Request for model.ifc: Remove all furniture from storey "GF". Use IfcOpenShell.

First a look at what the model holds.

```python
import ifcopenshell
import ifcopenshell.util.element

model = ifcopenshell.open("model.ifc")
print(model.schema)
storey = next(s for s in model.by_type("IfcBuildingStorey") if s.Name == "GF")
furniture = [e for e in ifcopenshell.util.element.get_decomposition(storey) if e.is_a("IfcFurnishingElement")]
seen = {}
for e in furniture:
    element_type = ifcopenshell.util.element.get_type(e)
    name = element_type.Name if element_type not in (None, e) else None
    seen[name] = seen.get(name, 0) + 1
for name, count in sorted(seen.items(), key=str):
    print(count, "x", name)
```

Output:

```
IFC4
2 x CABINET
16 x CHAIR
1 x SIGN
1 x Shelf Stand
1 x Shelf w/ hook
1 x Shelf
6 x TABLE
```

```python
import ifcopenshell
import ifcopenshell.api.root
import ifcopenshell.util.element

model = ifcopenshell.open("model.ifc")

storey = next(s for s in model.by_type("IfcBuildingStorey") if s.Name == "GF")
furniture = [e for e in ifcopenshell.util.element.get_decomposition(storey) if e.is_a("IfcFurnishingElement")]

for e in furniture:
    ifcopenshell.api.root.remove_product(model, product=e)
print(len(furniture), "removed")

model.write("model-out.ifc")
```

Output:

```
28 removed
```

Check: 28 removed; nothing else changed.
